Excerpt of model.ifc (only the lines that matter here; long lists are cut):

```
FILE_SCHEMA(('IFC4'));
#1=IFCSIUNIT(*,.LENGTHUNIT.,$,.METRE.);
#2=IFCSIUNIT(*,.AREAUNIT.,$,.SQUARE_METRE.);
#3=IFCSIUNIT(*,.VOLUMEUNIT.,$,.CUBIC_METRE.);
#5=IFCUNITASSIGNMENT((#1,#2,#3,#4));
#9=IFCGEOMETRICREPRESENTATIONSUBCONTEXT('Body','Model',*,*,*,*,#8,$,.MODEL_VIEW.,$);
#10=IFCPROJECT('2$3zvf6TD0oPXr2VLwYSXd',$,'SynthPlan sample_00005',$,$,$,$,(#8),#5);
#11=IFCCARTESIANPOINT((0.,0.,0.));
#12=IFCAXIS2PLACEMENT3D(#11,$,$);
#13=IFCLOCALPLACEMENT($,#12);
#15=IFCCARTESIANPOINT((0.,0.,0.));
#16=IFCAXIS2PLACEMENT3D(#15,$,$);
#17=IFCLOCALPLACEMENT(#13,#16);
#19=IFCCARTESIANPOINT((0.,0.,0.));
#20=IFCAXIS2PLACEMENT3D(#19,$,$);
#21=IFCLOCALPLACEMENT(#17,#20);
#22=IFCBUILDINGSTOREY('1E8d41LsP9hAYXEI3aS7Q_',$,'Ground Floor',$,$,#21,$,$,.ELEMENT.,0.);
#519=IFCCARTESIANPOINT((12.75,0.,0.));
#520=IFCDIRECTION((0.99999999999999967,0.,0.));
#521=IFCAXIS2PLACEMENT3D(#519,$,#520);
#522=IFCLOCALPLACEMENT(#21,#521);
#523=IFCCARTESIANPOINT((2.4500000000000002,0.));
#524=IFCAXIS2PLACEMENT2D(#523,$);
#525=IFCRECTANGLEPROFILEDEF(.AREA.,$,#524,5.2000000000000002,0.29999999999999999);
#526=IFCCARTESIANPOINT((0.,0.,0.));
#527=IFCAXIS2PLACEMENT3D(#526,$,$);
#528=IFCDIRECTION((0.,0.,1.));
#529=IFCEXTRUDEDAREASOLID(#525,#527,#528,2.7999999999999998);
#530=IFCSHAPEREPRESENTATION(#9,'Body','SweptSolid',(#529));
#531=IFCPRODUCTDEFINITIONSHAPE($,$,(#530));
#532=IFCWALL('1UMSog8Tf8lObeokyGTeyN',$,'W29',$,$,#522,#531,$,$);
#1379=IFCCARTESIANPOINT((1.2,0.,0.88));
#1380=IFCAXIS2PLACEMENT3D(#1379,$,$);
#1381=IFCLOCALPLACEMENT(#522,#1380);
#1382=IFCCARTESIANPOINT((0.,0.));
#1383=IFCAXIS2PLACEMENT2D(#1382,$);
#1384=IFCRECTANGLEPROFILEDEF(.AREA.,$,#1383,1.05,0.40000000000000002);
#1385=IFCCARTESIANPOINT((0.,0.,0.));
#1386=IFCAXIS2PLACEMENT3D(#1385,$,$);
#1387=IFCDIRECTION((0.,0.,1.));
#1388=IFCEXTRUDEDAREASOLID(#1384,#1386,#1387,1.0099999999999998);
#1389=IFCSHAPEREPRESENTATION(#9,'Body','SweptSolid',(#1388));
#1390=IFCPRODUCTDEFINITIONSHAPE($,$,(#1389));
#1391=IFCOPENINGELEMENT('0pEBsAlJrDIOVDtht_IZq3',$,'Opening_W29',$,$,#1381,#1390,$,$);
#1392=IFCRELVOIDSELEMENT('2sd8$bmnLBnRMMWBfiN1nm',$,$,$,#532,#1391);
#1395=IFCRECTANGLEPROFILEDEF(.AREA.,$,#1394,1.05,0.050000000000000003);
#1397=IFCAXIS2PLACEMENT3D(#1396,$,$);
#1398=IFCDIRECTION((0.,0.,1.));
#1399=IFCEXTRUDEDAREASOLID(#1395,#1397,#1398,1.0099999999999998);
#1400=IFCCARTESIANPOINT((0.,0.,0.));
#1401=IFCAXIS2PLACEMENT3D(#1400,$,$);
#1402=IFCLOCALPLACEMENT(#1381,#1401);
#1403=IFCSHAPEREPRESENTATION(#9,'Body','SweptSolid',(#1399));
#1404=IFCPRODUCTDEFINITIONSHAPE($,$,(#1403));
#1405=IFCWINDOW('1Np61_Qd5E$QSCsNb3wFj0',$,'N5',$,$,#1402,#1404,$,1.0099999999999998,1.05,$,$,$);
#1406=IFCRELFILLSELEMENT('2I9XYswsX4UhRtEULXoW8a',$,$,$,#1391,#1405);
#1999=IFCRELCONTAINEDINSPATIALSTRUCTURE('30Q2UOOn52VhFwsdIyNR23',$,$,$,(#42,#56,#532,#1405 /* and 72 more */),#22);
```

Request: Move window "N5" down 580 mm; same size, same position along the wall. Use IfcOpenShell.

```python
import numpy as np
import ifcopenshell
import ifcopenshell.api.geometry
import ifcopenshell.util.placement
import ifcopenshell.util.unit

model = ifcopenshell.open("model.ifc")
unit_scale = ifcopenshell.util.unit.calculate_unit_scale(model)

window = model.by_guid("1Np61_Qd5E$QSCsNb3wFj0")
opening = window.FillsVoids[0].RelatingOpeningElement
dz = -0.58

shift = np.array([0.0, 0.0, dz])
# The window is placed relative to its opening, so it follows when the opening moves.
matrix = ifcopenshell.util.placement.get_local_placement(opening.ObjectPlacement)
matrix[:3, 3] += shift
ifcopenshell.api.geometry.edit_object_placement(
    model, product=opening, matrix=matrix, is_si=False, should_transform_children=True
)

print(f"moved by {dz * unit_scale:+.3f} m")

model.write("model_updated.ifc")
```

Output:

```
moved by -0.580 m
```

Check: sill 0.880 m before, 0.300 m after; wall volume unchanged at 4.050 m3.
